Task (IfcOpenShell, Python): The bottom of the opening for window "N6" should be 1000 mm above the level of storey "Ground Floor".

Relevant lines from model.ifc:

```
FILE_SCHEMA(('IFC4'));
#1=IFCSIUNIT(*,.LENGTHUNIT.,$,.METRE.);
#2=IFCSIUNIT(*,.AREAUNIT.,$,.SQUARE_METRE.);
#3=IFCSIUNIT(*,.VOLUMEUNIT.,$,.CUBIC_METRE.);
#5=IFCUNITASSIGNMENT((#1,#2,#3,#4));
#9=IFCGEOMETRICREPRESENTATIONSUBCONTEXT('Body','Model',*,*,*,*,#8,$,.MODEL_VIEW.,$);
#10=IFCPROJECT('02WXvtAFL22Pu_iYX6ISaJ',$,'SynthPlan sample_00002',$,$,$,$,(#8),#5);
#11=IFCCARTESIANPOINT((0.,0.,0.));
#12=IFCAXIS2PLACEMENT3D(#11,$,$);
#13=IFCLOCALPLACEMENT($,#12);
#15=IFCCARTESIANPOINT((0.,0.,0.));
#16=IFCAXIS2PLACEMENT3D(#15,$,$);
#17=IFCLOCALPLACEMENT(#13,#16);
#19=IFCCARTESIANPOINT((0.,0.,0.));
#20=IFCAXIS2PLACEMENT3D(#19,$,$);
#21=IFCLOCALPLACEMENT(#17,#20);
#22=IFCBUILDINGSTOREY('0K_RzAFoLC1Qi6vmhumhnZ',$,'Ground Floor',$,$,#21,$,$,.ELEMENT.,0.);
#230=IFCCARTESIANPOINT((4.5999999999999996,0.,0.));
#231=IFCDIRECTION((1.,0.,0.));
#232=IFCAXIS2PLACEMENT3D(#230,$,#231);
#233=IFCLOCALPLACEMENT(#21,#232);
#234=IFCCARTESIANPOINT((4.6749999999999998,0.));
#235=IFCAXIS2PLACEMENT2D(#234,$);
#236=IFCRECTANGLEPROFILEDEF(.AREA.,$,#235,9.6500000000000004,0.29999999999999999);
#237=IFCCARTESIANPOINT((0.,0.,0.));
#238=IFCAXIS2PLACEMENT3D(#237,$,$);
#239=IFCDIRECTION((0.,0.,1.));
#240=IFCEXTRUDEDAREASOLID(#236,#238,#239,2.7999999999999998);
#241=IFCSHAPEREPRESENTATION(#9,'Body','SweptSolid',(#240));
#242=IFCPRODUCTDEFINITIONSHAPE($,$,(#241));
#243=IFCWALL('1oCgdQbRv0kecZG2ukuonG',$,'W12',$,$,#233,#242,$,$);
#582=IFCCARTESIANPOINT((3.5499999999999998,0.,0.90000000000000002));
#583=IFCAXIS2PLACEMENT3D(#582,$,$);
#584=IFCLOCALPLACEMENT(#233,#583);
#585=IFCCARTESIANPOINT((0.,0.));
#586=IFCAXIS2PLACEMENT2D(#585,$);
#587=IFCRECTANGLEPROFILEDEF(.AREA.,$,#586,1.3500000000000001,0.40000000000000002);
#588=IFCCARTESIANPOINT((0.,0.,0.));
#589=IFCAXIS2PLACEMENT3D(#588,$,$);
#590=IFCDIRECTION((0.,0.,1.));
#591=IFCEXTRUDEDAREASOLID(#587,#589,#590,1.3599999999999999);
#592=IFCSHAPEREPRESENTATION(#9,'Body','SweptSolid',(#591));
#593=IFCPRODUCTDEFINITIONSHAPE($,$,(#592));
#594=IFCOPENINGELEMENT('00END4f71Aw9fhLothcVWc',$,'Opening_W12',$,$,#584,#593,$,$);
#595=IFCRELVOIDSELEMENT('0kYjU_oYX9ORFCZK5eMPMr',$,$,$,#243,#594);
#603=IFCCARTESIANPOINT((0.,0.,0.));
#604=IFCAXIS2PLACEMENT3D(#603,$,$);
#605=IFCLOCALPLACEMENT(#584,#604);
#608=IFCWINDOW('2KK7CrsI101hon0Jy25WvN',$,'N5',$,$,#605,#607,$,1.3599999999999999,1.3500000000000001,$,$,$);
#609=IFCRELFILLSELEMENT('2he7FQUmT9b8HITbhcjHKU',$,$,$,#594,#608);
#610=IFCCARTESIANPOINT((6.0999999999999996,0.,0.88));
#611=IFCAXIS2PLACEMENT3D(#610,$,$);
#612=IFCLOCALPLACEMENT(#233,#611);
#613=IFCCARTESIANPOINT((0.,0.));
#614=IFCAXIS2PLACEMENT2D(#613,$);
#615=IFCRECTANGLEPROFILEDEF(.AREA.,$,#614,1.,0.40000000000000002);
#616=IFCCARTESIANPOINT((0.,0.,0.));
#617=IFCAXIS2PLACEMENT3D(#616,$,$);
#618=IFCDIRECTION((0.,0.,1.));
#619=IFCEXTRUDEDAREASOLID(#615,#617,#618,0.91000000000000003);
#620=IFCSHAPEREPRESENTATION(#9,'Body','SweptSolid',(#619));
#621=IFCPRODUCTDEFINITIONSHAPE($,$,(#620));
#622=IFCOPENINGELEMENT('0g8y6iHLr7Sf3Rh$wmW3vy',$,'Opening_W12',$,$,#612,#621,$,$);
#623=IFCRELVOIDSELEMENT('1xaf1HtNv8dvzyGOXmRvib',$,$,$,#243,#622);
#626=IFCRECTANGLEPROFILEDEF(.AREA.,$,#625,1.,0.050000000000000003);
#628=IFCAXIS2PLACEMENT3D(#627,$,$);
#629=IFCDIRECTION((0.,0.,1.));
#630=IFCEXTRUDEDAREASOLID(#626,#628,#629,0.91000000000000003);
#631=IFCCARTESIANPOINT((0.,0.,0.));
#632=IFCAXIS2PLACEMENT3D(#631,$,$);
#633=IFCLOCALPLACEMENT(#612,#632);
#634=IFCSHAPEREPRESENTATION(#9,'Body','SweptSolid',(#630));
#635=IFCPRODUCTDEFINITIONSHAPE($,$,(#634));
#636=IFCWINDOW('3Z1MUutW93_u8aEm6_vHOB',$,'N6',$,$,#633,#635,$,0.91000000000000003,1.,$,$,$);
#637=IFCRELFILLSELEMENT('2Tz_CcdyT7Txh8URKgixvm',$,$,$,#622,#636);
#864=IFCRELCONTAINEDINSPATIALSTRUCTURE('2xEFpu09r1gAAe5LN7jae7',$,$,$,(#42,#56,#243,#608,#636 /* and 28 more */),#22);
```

```python
import numpy as np
import ifcopenshell
import ifcopenshell.api.geometry
import ifcopenshell.geom
import ifcopenshell.util.element
import ifcopenshell.util.placement
import ifcopenshell.util.shape
import ifcopenshell.util.unit

model = ifcopenshell.open("model.ifc")
unit_scale = ifcopenshell.util.unit.calculate_unit_scale(model)

window = model.by_id(636)
opening = window.FillsVoids[0].RelatingOpeningElement
storey = ifcopenshell.util.element.get_container(window, ifc_class="IfcBuildingStorey")
level = ifcopenshell.util.placement.get_local_placement(storey.ObjectPlacement)[2, 3]

# The opening's origin need not be at the sill, so measure its lowest point.
shape = ifcopenshell.geom.create_shape(ifcopenshell.geom.settings(), opening)
bottom = ifcopenshell.util.shape.get_shape_bottom_elevation(shape, shape.geometry) / unit_scale
dz = level + 1.0 - bottom

shift = np.array([0.0, 0.0, dz])
# The window is placed relative to its opening, so it follows when the opening moves.
matrix = ifcopenshell.util.placement.get_local_placement(opening.ObjectPlacement)
matrix[:3, 3] += shift
ifcopenshell.api.geometry.edit_object_placement(
    model, product=opening, matrix=matrix, is_si=False, should_transform_children=True
)

print(f"moved by {dz * unit_scale:+.3f} m")

model.write("model_v2.ifc")
```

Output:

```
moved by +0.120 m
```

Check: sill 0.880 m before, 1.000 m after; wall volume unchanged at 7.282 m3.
